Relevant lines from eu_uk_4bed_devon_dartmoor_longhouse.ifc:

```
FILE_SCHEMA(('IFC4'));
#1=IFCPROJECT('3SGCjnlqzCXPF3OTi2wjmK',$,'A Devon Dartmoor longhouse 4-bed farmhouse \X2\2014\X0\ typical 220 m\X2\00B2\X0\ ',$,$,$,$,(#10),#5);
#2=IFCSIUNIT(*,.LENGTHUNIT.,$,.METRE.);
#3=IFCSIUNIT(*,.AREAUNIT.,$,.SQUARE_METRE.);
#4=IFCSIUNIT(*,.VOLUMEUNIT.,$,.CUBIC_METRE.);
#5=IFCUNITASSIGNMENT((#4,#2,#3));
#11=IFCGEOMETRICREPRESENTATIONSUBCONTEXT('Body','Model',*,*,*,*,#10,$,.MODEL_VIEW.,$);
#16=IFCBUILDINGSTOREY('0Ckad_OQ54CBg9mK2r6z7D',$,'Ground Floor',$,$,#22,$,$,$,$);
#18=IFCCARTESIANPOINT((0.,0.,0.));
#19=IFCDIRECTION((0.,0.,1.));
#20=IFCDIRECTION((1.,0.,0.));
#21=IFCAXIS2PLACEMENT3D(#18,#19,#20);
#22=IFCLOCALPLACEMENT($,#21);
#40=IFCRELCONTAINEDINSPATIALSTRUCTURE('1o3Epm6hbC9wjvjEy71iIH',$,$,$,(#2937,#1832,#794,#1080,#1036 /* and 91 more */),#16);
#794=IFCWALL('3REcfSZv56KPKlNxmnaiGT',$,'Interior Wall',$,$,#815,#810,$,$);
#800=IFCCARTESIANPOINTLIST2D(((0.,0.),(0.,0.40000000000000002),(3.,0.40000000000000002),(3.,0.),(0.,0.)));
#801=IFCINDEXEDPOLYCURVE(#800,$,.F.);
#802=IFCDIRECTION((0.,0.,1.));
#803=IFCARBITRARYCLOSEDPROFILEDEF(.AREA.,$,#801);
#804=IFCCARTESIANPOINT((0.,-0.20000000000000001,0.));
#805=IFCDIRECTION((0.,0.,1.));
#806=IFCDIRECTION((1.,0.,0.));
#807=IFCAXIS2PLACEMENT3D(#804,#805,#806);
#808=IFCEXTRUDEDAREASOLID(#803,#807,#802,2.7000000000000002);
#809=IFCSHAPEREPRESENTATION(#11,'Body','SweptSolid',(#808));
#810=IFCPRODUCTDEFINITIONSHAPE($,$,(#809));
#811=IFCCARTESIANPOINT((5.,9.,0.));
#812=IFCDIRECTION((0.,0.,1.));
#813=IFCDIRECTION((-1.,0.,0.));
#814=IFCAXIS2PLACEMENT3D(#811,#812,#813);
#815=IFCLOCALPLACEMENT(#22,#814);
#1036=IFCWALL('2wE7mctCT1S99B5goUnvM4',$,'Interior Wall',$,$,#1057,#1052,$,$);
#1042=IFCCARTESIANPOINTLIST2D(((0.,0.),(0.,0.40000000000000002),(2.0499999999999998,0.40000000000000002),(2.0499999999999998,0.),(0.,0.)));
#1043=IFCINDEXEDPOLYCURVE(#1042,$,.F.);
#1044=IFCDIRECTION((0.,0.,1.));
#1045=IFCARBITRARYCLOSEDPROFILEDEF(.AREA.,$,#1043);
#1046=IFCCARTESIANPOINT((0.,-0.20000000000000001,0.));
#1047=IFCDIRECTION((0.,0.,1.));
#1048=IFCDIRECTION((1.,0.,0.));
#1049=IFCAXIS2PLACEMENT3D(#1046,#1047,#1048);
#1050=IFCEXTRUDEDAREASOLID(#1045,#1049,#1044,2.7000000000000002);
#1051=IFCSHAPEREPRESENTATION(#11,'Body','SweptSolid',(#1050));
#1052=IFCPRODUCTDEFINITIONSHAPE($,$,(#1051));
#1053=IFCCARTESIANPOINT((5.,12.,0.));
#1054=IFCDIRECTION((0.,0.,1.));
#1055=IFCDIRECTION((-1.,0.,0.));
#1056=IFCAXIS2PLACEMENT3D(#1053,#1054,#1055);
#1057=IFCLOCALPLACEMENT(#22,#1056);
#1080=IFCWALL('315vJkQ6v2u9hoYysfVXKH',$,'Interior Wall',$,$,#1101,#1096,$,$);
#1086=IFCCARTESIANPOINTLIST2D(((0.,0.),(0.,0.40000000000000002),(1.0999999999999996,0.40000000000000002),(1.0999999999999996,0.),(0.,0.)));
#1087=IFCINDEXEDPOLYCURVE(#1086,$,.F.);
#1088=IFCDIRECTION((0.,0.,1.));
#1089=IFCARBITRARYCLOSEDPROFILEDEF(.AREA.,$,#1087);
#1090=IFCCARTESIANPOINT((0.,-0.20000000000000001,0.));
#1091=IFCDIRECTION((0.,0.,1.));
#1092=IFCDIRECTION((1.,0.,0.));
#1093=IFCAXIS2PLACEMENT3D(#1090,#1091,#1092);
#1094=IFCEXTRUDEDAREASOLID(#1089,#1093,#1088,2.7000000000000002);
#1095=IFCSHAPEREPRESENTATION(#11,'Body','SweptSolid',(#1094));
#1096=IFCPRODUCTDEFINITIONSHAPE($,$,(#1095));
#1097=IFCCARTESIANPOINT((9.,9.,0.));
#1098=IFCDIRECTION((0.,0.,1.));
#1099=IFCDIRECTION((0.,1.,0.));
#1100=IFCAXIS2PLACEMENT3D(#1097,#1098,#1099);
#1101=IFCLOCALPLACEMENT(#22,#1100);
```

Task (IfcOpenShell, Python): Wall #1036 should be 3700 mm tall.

```python
import ifcopenshell
import ifcopenshell.geom
import ifcopenshell.util.representation
import ifcopenshell.util.shape
import ifcopenshell.util.unit

model = ifcopenshell.open("eu_uk_4bed_devon_dartmoor_longhouse.ifc")
unit_scale = ifcopenshell.util.unit.calculate_unit_scale(model)
settings = ifcopenshell.geom.settings()


def volume(element):
    """Net volume in cubic metres, openings subtracted."""
    shape = ifcopenshell.geom.create_shape(settings, element)
    return ifcopenshell.util.shape.get_volume(shape.geometry)


wall = model.by_id(1036)
before = volume(wall)

body = ifcopenshell.util.representation.get_representation(wall, "Model", "Body")
solid = body.Items[0]
old_height = solid.Depth
solid.Depth = 3.7 / unit_scale
after = volume(wall)

print(f"height {old_height:g} -> {solid.Depth:g}, volume {before:.3f} -> {after:.3f} m3")

model.write("eu_uk_4bed_devon_dartmoor_longhouse_v2.ifc")
```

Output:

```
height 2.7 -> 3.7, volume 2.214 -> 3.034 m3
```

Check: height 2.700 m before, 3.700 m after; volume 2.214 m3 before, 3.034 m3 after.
